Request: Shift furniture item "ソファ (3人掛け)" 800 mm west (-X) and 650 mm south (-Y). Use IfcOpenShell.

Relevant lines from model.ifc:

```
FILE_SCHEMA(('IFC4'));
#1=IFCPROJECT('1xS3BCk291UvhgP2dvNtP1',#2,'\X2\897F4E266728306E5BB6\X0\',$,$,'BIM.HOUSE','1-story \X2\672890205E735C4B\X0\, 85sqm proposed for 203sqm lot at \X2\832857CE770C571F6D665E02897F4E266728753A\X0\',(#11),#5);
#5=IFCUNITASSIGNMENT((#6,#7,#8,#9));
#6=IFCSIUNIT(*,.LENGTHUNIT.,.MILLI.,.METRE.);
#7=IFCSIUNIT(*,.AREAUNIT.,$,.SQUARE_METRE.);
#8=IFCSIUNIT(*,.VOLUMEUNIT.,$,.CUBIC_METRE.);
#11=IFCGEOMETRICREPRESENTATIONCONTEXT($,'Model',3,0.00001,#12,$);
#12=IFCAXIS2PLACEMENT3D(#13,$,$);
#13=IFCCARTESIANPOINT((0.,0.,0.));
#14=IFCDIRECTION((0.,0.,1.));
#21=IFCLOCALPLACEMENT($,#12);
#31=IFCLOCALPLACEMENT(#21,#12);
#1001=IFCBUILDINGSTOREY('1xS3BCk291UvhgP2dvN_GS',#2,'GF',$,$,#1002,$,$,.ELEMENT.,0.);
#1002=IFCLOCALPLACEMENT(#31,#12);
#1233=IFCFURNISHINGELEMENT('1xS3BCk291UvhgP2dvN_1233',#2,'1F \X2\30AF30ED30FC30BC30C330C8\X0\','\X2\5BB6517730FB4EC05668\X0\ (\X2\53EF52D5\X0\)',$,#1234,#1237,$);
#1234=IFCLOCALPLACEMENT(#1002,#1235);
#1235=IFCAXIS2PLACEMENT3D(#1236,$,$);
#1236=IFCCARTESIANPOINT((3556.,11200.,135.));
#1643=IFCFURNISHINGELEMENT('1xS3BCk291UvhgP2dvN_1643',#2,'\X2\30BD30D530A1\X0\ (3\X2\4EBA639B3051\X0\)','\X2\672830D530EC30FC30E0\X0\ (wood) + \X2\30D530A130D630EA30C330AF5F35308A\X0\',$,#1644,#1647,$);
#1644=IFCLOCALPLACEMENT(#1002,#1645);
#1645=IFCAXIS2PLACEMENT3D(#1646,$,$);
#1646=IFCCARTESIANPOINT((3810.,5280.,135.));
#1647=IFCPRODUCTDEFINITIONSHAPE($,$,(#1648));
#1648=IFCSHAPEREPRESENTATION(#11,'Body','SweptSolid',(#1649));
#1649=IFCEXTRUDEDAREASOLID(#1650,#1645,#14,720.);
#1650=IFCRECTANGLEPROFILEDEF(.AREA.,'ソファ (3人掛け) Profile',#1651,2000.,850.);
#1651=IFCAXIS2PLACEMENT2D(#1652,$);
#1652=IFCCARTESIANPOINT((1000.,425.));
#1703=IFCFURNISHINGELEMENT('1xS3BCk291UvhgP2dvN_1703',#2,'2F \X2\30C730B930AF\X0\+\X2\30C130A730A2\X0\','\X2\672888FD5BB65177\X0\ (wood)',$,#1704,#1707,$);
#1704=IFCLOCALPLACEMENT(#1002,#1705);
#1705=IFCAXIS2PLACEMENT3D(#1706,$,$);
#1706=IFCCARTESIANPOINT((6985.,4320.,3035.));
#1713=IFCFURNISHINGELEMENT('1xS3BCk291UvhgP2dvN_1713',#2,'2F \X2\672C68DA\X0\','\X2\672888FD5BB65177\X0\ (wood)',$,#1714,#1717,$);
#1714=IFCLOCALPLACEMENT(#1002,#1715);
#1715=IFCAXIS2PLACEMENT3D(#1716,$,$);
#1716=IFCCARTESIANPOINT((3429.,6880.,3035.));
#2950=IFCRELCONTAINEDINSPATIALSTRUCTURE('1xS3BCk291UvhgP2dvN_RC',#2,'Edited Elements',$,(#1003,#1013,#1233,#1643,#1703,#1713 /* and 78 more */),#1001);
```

```python
import ifcopenshell
import ifcopenshell.api.geometry
import ifcopenshell.util.placement

model = ifcopenshell.open("model.ifc")

item = model.by_guid("1xS3BCk291UvhgP2dvN_1643")
matrix = ifcopenshell.util.placement.get_local_placement(item.ObjectPlacement)
matrix[0, 3] -= 800.0
matrix[1, 3] -= 650.0
ifcopenshell.api.geometry.edit_object_placement(model, product=item, matrix=matrix, is_si=False)

print(ifcopenshell.util.placement.get_local_placement(item.ObjectPlacement).round(3) + 0.0)

model.write("model_edited.ifc")
```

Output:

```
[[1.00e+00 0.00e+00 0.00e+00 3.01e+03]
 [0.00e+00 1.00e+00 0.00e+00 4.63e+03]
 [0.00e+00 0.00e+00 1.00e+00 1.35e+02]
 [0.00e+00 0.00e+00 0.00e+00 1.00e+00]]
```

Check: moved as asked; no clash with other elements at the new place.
